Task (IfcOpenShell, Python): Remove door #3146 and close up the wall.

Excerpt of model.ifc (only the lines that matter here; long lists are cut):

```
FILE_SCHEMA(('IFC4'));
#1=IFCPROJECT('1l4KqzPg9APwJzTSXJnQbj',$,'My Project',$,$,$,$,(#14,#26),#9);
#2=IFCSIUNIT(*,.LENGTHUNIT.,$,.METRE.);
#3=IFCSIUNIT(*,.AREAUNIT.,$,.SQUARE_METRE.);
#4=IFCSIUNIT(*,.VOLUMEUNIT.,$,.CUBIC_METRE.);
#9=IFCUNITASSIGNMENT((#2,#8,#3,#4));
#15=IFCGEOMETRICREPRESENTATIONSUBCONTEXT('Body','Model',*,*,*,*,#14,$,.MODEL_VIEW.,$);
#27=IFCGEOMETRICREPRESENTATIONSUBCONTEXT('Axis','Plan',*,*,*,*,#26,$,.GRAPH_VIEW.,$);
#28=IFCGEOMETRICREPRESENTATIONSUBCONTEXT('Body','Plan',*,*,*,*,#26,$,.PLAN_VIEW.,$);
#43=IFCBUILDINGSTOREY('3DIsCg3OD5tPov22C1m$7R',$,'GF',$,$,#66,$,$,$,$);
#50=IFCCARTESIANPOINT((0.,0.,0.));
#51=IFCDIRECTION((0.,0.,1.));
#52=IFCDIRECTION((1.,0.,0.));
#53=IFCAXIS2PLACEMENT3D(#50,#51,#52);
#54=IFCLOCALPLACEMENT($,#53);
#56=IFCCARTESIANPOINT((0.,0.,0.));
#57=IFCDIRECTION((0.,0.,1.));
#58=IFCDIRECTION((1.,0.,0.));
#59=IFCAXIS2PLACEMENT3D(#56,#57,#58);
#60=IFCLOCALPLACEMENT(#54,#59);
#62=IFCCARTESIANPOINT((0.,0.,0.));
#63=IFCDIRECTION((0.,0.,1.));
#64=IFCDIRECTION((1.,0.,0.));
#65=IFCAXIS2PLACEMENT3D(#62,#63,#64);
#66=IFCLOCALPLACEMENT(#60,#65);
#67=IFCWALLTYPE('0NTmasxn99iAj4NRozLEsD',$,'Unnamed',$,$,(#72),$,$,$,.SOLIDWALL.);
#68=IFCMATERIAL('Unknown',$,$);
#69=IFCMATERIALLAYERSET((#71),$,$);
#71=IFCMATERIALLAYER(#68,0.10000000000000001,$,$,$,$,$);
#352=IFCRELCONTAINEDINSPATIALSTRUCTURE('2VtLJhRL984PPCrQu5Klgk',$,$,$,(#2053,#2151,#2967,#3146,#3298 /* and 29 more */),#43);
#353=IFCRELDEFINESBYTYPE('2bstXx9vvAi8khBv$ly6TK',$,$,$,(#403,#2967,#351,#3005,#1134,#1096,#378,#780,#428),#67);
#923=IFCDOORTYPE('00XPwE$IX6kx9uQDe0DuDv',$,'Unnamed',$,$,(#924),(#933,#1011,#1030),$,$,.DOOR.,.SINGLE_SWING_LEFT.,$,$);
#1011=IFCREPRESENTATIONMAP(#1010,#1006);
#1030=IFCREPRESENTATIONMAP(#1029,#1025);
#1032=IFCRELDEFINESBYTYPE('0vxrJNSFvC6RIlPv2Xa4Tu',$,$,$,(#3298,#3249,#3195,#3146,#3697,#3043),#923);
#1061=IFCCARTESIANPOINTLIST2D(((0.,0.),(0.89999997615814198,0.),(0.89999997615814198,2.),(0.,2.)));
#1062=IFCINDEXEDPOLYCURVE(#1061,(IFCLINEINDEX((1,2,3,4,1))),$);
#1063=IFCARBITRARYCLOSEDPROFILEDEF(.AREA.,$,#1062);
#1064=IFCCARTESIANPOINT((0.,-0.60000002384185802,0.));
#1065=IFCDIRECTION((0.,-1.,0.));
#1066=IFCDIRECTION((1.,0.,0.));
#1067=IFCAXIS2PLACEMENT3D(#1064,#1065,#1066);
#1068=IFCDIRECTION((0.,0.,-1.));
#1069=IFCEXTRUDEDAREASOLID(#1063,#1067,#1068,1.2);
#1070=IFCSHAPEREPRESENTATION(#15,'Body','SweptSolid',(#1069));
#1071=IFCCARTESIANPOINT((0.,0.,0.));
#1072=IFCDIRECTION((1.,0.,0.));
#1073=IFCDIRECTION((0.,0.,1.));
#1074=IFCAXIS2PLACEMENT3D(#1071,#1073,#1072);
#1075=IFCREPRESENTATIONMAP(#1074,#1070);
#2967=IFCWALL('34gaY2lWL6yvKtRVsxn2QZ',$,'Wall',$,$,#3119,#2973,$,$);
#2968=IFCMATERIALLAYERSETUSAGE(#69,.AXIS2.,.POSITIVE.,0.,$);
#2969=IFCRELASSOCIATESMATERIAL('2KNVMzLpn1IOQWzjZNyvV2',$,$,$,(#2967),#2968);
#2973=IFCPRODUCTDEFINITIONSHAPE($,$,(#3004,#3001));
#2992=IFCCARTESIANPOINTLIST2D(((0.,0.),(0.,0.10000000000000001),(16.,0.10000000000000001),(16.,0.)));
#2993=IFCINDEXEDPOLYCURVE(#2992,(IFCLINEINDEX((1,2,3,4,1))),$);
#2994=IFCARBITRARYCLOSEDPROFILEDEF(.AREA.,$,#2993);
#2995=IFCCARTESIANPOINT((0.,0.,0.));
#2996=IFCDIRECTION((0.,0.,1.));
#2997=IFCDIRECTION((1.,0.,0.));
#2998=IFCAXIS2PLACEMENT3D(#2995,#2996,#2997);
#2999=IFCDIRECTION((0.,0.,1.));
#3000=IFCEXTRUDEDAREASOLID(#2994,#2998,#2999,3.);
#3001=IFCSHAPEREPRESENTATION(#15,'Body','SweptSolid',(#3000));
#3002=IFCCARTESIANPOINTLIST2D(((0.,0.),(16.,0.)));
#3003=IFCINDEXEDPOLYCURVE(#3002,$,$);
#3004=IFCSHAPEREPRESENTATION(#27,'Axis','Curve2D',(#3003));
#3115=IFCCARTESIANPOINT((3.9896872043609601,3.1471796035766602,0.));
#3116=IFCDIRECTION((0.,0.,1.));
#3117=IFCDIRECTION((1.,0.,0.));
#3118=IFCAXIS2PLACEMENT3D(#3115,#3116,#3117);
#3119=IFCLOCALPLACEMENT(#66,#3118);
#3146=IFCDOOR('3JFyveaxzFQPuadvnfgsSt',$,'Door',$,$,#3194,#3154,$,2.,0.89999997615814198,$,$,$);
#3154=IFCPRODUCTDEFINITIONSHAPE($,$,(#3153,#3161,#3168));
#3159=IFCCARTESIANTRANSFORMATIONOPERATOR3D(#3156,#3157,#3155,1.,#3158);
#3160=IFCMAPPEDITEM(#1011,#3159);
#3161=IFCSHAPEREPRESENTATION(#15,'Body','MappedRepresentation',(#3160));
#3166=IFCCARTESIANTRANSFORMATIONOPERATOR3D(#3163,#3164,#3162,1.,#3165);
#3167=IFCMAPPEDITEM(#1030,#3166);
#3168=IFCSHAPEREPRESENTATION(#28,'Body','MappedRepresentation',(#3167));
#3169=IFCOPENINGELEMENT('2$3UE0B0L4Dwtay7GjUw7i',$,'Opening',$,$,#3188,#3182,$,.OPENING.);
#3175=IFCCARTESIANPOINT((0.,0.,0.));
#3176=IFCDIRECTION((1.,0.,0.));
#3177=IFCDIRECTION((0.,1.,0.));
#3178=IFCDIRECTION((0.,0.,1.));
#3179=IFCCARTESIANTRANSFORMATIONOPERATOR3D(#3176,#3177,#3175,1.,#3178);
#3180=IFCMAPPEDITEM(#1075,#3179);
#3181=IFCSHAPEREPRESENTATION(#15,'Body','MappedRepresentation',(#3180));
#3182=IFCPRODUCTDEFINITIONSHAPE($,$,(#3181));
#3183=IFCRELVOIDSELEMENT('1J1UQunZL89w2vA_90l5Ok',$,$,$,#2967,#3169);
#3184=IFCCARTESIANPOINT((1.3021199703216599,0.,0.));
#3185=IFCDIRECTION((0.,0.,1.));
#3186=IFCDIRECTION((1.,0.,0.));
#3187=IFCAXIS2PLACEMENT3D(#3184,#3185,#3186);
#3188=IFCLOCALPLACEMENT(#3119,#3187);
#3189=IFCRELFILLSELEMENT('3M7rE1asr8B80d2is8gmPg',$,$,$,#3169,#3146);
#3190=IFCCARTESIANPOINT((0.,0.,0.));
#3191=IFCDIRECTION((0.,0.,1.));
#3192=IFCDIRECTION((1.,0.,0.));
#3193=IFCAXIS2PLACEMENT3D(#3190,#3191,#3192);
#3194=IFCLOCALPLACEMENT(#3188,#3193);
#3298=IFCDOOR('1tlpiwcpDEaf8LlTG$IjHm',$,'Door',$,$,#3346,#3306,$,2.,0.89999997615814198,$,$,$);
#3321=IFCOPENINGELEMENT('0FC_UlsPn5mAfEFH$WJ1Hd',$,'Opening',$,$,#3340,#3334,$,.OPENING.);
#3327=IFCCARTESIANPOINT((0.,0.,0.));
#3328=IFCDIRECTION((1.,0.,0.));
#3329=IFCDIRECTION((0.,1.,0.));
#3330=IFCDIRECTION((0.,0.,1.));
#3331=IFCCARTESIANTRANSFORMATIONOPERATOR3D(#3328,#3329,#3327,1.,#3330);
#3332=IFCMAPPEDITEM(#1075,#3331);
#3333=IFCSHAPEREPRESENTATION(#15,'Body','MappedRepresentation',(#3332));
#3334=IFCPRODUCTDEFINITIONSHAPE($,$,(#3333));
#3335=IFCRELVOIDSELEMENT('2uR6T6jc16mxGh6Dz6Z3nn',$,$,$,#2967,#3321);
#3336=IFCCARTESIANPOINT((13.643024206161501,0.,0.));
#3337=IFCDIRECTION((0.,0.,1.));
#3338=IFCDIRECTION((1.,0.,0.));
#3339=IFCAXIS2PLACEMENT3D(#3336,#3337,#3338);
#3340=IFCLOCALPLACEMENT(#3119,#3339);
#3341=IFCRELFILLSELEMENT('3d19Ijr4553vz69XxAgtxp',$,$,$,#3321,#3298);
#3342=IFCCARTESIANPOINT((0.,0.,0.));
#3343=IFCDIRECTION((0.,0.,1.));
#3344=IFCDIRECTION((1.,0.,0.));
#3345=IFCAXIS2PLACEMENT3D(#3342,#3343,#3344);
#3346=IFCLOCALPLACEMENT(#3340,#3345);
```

```python
import ifcopenshell
import ifcopenshell.api.feature
import ifcopenshell.api.root
import ifcopenshell.geom
import ifcopenshell.util.shape

model = ifcopenshell.open("model.ifc")
settings = ifcopenshell.geom.settings()


def volume(element):
    """Net volume in cubic metres, openings subtracted."""
    shape = ifcopenshell.geom.create_shape(settings, element)
    return ifcopenshell.util.shape.get_volume(shape.geometry)


door = model.by_id(3146)
opening = door.FillsVoids[0].RelatingOpeningElement
wall = opening.VoidsElements[0].RelatingBuildingElement
before = volume(wall)

ifcopenshell.api.root.remove_product(model, product=door)
ifcopenshell.api.feature.remove_feature(model, feature=opening)

after = volume(wall)

print(f"wall volume {before:.3f} -> {after:.3f} m3")

model.write("model_v2.ifc")
```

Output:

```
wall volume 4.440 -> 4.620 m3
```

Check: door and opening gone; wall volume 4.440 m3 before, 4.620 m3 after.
